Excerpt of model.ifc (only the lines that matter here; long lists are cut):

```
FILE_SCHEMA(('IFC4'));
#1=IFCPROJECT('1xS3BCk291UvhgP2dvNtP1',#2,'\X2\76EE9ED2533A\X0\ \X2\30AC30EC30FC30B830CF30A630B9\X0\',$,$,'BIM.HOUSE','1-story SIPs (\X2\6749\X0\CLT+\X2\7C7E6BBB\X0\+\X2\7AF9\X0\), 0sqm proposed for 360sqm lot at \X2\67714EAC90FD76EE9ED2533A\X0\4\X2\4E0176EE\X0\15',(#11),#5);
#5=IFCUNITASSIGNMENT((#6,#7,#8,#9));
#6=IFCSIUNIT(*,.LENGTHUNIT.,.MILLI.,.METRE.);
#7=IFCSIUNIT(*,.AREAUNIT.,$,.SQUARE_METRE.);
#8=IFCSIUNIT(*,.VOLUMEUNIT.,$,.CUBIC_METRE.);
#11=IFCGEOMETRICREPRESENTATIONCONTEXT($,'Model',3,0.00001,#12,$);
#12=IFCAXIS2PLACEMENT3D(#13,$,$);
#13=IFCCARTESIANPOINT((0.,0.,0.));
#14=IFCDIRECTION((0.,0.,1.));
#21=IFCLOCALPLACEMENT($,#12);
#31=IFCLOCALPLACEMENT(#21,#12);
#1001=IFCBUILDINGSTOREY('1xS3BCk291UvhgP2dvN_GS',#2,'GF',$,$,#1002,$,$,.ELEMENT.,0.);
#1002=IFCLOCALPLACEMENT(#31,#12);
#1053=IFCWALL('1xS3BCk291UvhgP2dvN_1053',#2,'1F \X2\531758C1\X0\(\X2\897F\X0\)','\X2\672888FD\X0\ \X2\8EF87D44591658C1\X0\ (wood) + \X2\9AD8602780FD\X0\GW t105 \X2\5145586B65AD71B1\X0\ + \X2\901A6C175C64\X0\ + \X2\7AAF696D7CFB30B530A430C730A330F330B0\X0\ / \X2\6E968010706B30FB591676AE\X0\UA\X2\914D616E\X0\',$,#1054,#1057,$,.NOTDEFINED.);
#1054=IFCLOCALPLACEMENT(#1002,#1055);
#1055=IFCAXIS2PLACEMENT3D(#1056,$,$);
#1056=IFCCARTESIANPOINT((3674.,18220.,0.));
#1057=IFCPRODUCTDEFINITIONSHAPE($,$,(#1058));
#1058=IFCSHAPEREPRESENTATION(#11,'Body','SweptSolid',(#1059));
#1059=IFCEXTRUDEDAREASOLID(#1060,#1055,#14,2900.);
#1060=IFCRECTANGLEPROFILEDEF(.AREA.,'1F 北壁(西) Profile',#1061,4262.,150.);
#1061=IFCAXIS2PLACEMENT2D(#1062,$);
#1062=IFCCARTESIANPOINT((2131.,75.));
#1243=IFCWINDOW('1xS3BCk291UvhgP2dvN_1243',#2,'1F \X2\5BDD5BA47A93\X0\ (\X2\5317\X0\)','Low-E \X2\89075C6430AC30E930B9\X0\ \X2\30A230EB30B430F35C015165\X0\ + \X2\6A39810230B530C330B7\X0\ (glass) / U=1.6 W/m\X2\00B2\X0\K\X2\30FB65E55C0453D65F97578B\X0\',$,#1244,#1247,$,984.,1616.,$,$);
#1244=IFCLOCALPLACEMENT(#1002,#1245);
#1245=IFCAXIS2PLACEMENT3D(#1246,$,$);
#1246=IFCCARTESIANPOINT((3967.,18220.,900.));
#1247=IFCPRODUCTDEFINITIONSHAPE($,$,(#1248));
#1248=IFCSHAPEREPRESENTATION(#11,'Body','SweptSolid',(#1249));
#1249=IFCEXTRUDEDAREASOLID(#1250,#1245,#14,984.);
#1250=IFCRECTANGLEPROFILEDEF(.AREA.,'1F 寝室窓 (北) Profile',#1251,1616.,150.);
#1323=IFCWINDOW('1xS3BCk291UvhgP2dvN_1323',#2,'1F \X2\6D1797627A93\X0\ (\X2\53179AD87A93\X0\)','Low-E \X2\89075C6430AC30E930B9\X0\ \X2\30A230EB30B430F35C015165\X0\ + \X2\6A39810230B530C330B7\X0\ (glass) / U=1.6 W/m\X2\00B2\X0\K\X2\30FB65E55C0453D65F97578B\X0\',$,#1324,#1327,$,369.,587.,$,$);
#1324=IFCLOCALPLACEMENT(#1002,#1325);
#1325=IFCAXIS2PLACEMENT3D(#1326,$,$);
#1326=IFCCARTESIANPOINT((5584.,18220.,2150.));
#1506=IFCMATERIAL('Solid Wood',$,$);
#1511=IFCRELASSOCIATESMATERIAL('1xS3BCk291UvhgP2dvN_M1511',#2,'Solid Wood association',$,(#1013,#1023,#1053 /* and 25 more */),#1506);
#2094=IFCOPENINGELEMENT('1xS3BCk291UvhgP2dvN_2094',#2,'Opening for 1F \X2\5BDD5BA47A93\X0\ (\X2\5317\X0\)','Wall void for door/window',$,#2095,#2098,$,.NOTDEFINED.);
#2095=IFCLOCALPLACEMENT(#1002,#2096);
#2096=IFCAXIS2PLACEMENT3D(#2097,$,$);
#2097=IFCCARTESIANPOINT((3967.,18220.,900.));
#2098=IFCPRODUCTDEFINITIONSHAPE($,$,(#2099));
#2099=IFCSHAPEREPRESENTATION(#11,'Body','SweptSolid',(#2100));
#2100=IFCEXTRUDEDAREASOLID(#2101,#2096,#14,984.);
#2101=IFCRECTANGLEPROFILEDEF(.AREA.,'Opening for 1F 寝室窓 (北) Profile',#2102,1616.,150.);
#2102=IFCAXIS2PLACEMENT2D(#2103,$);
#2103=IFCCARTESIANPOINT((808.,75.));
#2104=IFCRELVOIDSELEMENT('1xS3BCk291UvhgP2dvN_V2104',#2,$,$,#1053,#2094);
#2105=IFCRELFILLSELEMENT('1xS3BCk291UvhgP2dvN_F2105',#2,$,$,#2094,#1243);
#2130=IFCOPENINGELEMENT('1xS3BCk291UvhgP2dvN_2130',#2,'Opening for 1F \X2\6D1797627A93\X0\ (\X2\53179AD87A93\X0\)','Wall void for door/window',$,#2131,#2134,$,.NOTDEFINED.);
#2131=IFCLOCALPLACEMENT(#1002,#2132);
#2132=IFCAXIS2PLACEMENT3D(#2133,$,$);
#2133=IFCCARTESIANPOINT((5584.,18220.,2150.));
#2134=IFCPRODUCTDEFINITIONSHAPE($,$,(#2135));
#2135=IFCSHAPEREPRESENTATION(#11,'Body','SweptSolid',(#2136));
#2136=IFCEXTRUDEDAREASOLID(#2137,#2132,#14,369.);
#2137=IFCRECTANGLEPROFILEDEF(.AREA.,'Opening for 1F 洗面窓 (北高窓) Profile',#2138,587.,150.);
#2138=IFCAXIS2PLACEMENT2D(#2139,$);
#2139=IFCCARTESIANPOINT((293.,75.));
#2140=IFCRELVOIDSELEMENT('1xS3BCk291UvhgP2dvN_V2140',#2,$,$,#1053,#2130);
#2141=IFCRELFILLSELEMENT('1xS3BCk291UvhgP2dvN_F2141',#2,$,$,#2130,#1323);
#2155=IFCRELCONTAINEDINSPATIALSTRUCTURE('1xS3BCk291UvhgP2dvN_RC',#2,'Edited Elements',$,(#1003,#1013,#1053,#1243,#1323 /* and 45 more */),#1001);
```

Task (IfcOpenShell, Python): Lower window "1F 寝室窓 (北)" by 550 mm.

```python
import numpy as np
import ifcopenshell
import ifcopenshell.api.geometry
import ifcopenshell.util.placement
import ifcopenshell.util.unit

model = ifcopenshell.open("model.ifc")
unit_scale = ifcopenshell.util.unit.calculate_unit_scale(model)

window = model.by_guid("1xS3BCk291UvhgP2dvN_1243")
opening = window.FillsVoids[0].RelatingOpeningElement
dz = -0.55 / unit_scale

shift = np.array([0.0, 0.0, dz])
# The window is not placed relative to its opening, so move both.
for product in (opening, window):
    matrix = ifcopenshell.util.placement.get_local_placement(product.ObjectPlacement)
    matrix[:3, 3] += shift
    ifcopenshell.api.geometry.edit_object_placement(model, product=product, matrix=matrix, is_si=False)

print(f"moved by {dz * unit_scale:+.3f} m")

model.write("model_v2.ifc")
```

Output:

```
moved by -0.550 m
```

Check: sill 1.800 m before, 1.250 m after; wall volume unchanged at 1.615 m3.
